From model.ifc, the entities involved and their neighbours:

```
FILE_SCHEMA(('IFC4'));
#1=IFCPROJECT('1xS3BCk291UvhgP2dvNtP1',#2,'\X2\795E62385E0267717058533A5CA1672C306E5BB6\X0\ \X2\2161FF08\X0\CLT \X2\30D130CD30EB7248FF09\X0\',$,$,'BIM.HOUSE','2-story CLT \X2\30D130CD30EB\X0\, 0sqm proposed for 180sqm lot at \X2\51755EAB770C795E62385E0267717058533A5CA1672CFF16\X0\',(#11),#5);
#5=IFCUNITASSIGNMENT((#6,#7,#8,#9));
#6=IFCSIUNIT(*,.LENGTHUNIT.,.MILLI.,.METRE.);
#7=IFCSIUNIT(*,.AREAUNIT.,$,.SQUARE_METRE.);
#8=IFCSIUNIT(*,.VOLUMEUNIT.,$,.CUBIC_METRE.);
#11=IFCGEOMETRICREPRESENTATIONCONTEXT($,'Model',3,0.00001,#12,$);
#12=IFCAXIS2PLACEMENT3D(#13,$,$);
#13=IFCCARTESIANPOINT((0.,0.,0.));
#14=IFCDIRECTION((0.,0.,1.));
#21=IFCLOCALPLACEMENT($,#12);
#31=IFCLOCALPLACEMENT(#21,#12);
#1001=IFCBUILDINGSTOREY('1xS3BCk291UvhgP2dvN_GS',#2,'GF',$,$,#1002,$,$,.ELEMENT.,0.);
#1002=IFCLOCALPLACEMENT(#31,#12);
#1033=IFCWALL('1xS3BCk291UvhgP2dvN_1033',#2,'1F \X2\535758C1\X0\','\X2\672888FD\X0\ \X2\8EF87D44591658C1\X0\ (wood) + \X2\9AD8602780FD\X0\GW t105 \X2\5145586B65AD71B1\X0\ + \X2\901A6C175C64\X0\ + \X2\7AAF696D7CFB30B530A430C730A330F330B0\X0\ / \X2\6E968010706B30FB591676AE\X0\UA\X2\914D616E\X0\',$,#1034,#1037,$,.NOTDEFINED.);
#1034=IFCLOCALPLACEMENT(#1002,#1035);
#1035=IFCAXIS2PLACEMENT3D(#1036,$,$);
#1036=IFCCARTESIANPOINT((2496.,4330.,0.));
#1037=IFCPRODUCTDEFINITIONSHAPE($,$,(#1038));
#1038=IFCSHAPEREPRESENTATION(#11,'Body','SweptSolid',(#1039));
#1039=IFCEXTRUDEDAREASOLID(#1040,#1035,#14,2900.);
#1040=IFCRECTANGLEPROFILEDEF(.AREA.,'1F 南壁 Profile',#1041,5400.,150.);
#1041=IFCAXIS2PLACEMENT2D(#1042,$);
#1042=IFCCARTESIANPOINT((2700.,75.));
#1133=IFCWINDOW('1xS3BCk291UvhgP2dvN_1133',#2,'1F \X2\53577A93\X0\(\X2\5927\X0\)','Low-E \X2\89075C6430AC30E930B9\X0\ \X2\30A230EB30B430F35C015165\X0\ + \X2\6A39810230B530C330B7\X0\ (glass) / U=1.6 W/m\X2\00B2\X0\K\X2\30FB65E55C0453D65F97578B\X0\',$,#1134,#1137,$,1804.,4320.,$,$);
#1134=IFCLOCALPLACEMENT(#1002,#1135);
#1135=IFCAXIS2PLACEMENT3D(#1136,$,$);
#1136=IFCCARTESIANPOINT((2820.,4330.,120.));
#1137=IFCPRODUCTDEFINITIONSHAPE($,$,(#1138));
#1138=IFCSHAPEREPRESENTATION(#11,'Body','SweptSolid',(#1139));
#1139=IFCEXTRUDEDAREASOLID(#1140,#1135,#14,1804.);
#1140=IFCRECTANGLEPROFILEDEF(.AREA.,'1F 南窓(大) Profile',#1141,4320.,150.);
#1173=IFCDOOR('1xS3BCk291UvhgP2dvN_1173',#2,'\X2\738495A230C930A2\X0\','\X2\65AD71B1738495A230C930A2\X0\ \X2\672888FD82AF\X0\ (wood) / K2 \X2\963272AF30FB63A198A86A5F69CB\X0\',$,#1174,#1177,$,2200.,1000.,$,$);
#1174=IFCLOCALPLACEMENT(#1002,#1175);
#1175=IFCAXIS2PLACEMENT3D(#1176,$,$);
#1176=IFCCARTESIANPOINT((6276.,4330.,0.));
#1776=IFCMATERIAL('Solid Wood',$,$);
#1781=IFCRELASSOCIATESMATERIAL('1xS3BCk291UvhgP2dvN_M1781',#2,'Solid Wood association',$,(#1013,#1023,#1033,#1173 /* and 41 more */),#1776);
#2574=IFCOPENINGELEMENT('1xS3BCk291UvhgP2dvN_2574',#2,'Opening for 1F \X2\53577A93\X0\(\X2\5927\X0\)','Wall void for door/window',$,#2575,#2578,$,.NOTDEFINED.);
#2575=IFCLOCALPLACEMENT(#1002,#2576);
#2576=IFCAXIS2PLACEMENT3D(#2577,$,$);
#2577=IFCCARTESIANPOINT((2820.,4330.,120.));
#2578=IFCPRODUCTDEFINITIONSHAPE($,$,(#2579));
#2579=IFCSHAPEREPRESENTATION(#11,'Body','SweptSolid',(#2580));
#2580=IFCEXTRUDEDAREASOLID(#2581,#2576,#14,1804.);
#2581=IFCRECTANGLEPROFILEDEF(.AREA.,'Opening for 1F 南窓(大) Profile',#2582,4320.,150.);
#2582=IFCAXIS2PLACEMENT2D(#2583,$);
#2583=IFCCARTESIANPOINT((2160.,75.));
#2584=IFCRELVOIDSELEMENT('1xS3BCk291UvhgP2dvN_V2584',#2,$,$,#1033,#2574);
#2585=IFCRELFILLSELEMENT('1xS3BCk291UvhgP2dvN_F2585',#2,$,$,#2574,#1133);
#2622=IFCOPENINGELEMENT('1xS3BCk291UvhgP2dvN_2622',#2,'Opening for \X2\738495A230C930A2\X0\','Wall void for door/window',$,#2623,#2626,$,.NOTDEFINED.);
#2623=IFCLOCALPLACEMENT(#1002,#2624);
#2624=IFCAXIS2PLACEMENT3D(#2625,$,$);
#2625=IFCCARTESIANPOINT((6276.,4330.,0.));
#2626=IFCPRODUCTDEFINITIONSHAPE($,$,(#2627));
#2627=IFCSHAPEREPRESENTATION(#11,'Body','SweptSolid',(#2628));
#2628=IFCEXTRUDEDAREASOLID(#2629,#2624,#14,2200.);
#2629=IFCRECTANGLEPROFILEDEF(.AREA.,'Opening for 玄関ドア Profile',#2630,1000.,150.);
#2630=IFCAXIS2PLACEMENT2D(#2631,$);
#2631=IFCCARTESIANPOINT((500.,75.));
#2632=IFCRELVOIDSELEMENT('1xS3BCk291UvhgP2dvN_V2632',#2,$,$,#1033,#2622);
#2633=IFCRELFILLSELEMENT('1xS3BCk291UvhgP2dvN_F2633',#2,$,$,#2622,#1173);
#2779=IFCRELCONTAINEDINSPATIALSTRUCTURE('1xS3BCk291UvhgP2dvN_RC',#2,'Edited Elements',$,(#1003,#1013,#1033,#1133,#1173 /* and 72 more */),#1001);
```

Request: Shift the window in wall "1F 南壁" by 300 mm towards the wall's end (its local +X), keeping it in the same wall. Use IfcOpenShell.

```python
import ifcopenshell
import ifcopenshell.api.geometry
import ifcopenshell.util.placement

model = ifcopenshell.open("model.ifc")

window = model.by_guid("1xS3BCk291UvhgP2dvN_1133")
opening = window.FillsVoids[0].RelatingOpeningElement
wall = opening.VoidsElements[0].RelatingBuildingElement

wall_matrix = ifcopenshell.util.placement.get_local_placement(wall.ObjectPlacement)
shift = wall_matrix[:3, 0] * 300.0
before = ifcopenshell.util.placement.get_local_placement(window.ObjectPlacement)[:3, 3].copy()

# The window is not placed relative to its opening, so move both.
for product in (opening, window):
    matrix = ifcopenshell.util.placement.get_local_placement(product.ObjectPlacement)
    matrix[:3, 3] += shift
    ifcopenshell.api.geometry.edit_object_placement(model, product=product, matrix=matrix, is_si=False)

after = ifcopenshell.util.placement.get_local_placement(window.ObjectPlacement)[:3, 3]
print("window moved by", (after - before).round(3) + 0.0)

model.write("model_v2.ifc")
```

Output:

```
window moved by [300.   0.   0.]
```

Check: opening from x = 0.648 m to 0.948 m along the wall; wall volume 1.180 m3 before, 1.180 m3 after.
